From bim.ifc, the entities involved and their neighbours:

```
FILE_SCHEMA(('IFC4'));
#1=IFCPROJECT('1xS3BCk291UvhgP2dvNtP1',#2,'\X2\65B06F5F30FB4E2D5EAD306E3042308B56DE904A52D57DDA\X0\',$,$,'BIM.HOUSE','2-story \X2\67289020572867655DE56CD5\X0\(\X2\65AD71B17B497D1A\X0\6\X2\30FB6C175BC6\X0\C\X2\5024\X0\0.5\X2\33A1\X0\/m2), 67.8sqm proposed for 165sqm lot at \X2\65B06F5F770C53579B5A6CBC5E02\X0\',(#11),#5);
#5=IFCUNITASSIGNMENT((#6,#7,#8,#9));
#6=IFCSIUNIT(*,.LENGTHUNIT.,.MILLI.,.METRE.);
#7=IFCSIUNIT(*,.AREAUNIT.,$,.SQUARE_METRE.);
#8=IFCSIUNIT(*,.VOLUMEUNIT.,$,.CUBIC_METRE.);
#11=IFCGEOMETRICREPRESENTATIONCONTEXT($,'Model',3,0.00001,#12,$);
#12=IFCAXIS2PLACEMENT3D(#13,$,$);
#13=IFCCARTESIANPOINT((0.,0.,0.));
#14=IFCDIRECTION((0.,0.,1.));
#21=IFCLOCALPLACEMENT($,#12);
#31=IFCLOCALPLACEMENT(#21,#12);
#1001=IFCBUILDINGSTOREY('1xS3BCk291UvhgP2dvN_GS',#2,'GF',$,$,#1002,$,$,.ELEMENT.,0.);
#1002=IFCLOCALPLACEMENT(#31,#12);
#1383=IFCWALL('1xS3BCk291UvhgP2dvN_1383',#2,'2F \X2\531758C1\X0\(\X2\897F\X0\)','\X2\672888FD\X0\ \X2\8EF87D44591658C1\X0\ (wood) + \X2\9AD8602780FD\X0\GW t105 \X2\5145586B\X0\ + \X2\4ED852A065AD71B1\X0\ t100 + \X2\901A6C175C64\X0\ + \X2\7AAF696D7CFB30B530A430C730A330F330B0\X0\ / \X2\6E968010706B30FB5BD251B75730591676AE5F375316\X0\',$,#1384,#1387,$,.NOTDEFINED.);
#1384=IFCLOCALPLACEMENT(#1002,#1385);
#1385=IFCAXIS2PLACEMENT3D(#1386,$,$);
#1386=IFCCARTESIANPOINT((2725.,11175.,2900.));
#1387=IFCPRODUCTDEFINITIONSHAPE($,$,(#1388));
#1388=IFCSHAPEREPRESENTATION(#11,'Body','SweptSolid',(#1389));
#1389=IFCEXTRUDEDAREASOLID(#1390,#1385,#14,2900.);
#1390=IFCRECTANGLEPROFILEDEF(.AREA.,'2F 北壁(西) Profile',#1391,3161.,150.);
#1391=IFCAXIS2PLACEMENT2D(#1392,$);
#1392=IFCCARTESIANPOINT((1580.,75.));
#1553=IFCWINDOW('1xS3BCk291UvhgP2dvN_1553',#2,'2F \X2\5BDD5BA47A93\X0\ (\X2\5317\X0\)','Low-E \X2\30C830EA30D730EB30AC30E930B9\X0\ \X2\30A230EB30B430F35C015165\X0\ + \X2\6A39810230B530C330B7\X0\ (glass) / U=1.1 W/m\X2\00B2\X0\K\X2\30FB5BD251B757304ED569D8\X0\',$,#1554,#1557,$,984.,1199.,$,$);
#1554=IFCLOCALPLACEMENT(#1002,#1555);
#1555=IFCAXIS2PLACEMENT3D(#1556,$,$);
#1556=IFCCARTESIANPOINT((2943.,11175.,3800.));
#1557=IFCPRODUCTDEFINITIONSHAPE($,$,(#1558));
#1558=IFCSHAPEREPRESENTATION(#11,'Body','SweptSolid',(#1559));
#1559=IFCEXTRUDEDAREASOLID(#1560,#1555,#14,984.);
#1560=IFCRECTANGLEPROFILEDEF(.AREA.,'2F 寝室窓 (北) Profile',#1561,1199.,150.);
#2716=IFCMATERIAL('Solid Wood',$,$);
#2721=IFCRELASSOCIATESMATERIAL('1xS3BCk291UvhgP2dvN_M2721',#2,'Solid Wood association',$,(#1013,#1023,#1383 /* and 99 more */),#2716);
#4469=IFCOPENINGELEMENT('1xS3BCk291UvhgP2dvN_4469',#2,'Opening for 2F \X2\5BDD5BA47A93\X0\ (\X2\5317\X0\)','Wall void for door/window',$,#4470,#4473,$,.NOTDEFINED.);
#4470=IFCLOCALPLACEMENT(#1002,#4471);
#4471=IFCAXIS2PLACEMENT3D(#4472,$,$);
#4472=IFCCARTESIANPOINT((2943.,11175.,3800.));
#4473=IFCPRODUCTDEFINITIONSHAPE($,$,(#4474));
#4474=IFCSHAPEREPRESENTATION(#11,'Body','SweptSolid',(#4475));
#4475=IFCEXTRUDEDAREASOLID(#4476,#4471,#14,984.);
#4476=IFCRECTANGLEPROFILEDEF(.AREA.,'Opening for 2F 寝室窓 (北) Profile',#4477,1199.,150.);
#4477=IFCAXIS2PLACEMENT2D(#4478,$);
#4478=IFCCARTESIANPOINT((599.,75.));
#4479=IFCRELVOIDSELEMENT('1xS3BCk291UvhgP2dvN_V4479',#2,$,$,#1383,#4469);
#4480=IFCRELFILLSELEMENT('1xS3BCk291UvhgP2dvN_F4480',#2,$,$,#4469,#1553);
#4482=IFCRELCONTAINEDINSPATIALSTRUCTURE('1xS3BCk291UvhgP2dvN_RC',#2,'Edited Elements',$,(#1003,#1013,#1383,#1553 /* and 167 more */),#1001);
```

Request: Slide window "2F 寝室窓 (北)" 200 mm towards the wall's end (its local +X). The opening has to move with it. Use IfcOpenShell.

```python
import ifcopenshell
import ifcopenshell.api.geometry
import ifcopenshell.util.placement
import ifcopenshell.util.unit

model = ifcopenshell.open("bim.ifc")
unit_scale = ifcopenshell.util.unit.calculate_unit_scale(model)

window = model.by_id(1553)
opening = window.FillsVoids[0].RelatingOpeningElement
wall = opening.VoidsElements[0].RelatingBuildingElement

wall_matrix = ifcopenshell.util.placement.get_local_placement(wall.ObjectPlacement)
shift = wall_matrix[:3, 0] * 0.2 / unit_scale
before = ifcopenshell.util.placement.get_local_placement(window.ObjectPlacement)[:3, 3].copy()

# The window is not placed relative to its opening, so move both.
for product in (opening, window):
    matrix = ifcopenshell.util.placement.get_local_placement(product.ObjectPlacement)
    matrix[:3, 3] += shift
    ifcopenshell.api.geometry.edit_object_placement(model, product=product, matrix=matrix, is_si=False)

after = ifcopenshell.util.placement.get_local_placement(window.ObjectPlacement)[:3, 3]
print("window moved by", (after - before).round(3) + 0.0)

model.write("bim_updated.ifc")
```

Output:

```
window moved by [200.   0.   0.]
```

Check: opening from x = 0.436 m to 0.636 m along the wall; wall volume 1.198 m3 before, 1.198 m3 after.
